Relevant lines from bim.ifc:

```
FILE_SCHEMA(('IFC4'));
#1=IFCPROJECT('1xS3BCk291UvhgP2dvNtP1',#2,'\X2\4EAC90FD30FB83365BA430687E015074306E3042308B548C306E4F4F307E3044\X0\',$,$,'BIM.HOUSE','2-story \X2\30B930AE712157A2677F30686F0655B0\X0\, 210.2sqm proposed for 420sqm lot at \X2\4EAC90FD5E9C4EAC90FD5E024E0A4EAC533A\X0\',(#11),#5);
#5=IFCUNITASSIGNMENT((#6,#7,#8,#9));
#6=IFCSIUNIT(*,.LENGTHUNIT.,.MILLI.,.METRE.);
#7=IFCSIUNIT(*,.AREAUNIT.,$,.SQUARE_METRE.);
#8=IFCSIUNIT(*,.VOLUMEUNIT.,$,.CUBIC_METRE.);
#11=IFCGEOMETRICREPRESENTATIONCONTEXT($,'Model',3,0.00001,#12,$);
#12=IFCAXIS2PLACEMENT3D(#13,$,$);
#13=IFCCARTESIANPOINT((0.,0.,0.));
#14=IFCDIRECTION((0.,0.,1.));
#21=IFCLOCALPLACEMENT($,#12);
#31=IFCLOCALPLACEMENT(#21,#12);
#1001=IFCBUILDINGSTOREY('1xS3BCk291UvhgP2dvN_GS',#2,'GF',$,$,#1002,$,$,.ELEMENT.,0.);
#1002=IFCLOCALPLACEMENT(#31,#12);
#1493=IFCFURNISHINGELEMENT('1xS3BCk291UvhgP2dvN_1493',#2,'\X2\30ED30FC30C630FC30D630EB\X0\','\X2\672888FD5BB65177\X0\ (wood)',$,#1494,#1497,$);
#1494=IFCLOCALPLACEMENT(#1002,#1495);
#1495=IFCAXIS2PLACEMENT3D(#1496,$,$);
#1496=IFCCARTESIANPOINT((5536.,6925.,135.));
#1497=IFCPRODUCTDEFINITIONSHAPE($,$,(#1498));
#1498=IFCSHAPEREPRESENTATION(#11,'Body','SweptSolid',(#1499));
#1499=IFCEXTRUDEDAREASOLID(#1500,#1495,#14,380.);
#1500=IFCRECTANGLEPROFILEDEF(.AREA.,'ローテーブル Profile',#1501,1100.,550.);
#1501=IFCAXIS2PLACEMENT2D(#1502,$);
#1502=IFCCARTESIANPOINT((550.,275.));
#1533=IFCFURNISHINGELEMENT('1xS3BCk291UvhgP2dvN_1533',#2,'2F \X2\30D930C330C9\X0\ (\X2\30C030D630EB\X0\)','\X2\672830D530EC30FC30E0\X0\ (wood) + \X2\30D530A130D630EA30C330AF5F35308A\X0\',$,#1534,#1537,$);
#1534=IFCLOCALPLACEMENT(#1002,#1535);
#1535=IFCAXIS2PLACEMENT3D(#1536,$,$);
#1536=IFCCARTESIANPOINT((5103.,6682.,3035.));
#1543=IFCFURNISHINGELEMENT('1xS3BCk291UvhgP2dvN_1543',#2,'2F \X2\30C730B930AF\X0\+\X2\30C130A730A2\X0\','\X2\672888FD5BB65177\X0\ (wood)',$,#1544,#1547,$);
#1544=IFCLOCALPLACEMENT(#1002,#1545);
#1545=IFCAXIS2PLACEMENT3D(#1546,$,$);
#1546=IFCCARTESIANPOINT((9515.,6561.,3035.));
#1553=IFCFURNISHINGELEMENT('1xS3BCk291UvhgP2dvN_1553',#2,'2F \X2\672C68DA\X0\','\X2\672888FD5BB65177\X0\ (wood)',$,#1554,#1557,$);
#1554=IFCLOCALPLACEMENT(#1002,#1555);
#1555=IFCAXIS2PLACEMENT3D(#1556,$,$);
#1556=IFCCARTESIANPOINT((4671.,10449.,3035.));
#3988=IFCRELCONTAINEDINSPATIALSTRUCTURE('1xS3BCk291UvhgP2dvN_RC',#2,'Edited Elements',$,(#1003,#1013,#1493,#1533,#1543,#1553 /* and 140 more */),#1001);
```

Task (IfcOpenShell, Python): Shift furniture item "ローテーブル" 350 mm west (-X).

```python
import ifcopenshell
import ifcopenshell.api.geometry
import ifcopenshell.util.placement

model = ifcopenshell.open("bim.ifc")

item = model.by_guid("1xS3BCk291UvhgP2dvN_1493")
matrix = ifcopenshell.util.placement.get_local_placement(item.ObjectPlacement)
matrix[0, 3] -= 350.0
ifcopenshell.api.geometry.edit_object_placement(model, product=item, matrix=matrix, is_si=False)

print(ifcopenshell.util.placement.get_local_placement(item.ObjectPlacement).round(3) + 0.0)

model.write("bim_v2.ifc")
```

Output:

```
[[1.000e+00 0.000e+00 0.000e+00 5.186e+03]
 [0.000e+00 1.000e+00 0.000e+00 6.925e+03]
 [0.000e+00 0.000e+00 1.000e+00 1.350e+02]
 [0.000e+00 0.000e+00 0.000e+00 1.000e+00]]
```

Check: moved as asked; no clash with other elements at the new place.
